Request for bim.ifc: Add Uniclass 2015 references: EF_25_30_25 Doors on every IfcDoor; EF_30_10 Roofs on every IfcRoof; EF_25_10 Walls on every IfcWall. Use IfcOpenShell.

First a look at what the model holds.

```python
import ifcopenshell

model = ifcopenshell.open("bim.ifc")
print(model.schema)
print("classifications:", [c.Name for c in model.by_type("IfcClassification")])
for ifc_class in ("IfcDoor", "IfcRoof", "IfcStair", "IfcWall", "IfcWindow"):
    print(ifc_class, len(model.by_type(ifc_class)))
```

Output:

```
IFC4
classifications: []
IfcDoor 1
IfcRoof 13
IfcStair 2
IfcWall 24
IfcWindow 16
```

```python
import ifcopenshell
import ifcopenshell.api.classification

model = ifcopenshell.open("bim.ifc")

system = ifcopenshell.api.classification.add_classification(model, classification="Uniclass 2015")

codes = {
    "IfcDoor": ("EF_25_30_25", "Doors"),
    "IfcRoof": ("EF_30_10", "Roofs"),
    "IfcWall": ("EF_25_10", "Walls"),
}
for ifc_class, (code, name) in codes.items():
    products = model.by_type(ifc_class)
    ifcopenshell.api.classification.add_reference(
        model, products=products, classification=system, identification=code, name=name
    )
    print(code, len(products))

model.write("bim_rev.ifc")
```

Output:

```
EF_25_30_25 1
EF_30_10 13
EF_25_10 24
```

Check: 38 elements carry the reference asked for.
